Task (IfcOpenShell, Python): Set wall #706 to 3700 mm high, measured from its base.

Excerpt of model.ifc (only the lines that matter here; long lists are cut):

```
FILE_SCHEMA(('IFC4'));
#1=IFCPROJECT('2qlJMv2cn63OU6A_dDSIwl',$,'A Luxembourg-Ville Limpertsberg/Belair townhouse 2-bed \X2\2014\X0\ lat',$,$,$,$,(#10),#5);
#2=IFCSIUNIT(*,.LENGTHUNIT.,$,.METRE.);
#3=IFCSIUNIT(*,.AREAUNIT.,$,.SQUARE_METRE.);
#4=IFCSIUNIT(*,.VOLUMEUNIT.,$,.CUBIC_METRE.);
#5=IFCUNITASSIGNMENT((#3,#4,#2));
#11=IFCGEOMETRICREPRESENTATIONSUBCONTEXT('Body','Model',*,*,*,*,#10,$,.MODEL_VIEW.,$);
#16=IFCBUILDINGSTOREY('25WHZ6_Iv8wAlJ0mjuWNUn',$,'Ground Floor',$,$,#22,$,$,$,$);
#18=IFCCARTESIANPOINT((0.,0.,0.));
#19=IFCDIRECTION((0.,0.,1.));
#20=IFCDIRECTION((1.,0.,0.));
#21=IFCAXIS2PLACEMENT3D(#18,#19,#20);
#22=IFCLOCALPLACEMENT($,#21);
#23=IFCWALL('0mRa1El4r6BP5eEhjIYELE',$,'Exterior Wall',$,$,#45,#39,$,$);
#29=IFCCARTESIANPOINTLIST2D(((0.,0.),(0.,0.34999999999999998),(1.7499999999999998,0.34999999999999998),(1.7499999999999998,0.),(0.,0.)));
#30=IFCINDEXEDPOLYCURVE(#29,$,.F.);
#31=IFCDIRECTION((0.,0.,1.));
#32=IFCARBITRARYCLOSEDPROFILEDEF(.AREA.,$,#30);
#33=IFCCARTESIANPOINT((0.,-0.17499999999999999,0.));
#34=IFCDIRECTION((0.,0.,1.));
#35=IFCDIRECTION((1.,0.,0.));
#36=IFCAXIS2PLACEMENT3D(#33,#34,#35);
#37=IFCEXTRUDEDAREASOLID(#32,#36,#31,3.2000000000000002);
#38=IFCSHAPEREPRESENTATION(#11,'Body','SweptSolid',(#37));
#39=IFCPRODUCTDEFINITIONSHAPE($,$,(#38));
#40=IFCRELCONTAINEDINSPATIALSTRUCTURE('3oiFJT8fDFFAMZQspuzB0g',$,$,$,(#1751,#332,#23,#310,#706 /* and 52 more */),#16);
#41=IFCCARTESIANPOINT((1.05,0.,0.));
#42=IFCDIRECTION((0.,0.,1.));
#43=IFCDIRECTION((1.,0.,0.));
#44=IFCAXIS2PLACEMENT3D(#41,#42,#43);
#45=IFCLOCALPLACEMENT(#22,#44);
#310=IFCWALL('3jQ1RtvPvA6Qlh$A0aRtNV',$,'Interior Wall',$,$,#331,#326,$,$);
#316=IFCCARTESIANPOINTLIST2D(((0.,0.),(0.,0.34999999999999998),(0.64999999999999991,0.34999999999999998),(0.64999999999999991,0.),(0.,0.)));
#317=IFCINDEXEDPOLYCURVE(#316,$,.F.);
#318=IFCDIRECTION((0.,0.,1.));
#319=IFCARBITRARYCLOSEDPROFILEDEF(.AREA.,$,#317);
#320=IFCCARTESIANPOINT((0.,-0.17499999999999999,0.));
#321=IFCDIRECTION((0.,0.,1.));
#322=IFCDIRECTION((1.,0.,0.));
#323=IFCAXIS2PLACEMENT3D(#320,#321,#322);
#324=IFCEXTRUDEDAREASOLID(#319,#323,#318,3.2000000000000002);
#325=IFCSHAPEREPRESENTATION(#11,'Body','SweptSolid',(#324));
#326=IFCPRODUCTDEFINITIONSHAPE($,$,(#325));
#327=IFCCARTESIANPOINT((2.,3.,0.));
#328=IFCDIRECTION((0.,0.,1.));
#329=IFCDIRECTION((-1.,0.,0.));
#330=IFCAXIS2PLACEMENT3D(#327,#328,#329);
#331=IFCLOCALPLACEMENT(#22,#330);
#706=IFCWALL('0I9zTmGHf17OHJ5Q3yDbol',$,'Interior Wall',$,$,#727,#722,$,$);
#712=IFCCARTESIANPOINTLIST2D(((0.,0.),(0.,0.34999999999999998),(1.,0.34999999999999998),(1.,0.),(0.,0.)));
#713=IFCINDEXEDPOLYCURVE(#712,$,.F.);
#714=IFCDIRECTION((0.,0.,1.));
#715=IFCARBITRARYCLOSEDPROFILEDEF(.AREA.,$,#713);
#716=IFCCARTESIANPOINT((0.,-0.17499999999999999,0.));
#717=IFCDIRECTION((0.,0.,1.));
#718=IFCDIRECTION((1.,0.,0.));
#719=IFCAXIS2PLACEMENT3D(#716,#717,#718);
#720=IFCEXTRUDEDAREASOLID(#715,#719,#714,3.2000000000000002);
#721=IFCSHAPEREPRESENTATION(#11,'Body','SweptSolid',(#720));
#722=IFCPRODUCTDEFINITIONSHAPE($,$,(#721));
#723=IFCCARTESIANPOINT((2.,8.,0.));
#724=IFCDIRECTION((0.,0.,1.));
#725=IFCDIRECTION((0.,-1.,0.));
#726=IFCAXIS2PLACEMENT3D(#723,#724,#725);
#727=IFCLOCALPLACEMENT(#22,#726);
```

```python
import ifcopenshell
import ifcopenshell.geom
import ifcopenshell.util.representation
import ifcopenshell.util.shape
import ifcopenshell.util.unit

model = ifcopenshell.open("model.ifc")
unit_scale = ifcopenshell.util.unit.calculate_unit_scale(model)
settings = ifcopenshell.geom.settings()


def volume(element):
    """Net volume in cubic metres, openings subtracted."""
    shape = ifcopenshell.geom.create_shape(settings, element)
    return ifcopenshell.util.shape.get_volume(shape.geometry)


wall = model.by_guid("0I9zTmGHf17OHJ5Q3yDbol")
before = volume(wall)

body = ifcopenshell.util.representation.get_representation(wall, "Model", "Body")
solid = body.Items[0]
old_height = solid.Depth
solid.Depth = 3.7 / unit_scale
after = volume(wall)

print(f"height {old_height:g} -> {solid.Depth:g}, volume {before:.3f} -> {after:.3f} m3")

model.write("model_edited.ifc")
```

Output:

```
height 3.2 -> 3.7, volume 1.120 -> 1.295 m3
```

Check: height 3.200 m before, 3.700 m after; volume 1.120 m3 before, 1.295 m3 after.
